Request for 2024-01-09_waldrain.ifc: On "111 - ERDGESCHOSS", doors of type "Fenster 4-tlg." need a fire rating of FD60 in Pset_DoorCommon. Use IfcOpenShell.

First a look at what the model holds.

```python
import ifcopenshell
import ifcopenshell.util.element

model = ifcopenshell.open("2024-01-09_waldrain.ifc")
print(model.schema)
storey = next(s for s in model.by_type("IfcBuildingStorey") if s.Name == "111 - ERDGESCHOSS")
doors = [e for e in ifcopenshell.util.element.get_decomposition(storey) if e.is_a("IfcDoor")]
seen = {}
for e in doors:
    element_type = ifcopenshell.util.element.get_type(e)
    key = (element_type.Name if element_type != e and element_type else None, ifcopenshell.util.element.get_pset(e, "Pset_DoorCommon", "FireRating"))
    seen[key] = seen.get(key, 0) + 1
for (name, value), count in sorted(seen.items(), key=str):
    print(count, "x", name, "|", value)
```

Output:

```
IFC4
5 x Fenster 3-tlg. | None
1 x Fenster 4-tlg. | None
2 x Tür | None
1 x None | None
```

```python
import ifcopenshell
import ifcopenshell.api.pset
import ifcopenshell.util.element

model = ifcopenshell.open("2024-01-09_waldrain.ifc")

storey = next(s for s in model.by_type("IfcBuildingStorey") if s.Name == "111 - ERDGESCHOSS")
doors = [e for e in ifcopenshell.util.element.get_decomposition(storey) if e.is_a("IfcDoor")]

count = 0
for e in doors:
    element_type = ifcopenshell.util.element.get_type(e)
    if element_type in (None, e) or element_type.Name != "Fenster 4-tlg.":
        continue
    # add_pset returns the element's existing set when there is one.
    pset = ifcopenshell.api.pset.add_pset(model, product=e, name="Pset_DoorCommon")
    ifcopenshell.api.pset.edit_pset(model, pset=pset, properties={"FireRating": "FD60"})
    count += 1

print(count, "doors updated")

model.write("2024-01-09_waldrain_updated.ifc")
```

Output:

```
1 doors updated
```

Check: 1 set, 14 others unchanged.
